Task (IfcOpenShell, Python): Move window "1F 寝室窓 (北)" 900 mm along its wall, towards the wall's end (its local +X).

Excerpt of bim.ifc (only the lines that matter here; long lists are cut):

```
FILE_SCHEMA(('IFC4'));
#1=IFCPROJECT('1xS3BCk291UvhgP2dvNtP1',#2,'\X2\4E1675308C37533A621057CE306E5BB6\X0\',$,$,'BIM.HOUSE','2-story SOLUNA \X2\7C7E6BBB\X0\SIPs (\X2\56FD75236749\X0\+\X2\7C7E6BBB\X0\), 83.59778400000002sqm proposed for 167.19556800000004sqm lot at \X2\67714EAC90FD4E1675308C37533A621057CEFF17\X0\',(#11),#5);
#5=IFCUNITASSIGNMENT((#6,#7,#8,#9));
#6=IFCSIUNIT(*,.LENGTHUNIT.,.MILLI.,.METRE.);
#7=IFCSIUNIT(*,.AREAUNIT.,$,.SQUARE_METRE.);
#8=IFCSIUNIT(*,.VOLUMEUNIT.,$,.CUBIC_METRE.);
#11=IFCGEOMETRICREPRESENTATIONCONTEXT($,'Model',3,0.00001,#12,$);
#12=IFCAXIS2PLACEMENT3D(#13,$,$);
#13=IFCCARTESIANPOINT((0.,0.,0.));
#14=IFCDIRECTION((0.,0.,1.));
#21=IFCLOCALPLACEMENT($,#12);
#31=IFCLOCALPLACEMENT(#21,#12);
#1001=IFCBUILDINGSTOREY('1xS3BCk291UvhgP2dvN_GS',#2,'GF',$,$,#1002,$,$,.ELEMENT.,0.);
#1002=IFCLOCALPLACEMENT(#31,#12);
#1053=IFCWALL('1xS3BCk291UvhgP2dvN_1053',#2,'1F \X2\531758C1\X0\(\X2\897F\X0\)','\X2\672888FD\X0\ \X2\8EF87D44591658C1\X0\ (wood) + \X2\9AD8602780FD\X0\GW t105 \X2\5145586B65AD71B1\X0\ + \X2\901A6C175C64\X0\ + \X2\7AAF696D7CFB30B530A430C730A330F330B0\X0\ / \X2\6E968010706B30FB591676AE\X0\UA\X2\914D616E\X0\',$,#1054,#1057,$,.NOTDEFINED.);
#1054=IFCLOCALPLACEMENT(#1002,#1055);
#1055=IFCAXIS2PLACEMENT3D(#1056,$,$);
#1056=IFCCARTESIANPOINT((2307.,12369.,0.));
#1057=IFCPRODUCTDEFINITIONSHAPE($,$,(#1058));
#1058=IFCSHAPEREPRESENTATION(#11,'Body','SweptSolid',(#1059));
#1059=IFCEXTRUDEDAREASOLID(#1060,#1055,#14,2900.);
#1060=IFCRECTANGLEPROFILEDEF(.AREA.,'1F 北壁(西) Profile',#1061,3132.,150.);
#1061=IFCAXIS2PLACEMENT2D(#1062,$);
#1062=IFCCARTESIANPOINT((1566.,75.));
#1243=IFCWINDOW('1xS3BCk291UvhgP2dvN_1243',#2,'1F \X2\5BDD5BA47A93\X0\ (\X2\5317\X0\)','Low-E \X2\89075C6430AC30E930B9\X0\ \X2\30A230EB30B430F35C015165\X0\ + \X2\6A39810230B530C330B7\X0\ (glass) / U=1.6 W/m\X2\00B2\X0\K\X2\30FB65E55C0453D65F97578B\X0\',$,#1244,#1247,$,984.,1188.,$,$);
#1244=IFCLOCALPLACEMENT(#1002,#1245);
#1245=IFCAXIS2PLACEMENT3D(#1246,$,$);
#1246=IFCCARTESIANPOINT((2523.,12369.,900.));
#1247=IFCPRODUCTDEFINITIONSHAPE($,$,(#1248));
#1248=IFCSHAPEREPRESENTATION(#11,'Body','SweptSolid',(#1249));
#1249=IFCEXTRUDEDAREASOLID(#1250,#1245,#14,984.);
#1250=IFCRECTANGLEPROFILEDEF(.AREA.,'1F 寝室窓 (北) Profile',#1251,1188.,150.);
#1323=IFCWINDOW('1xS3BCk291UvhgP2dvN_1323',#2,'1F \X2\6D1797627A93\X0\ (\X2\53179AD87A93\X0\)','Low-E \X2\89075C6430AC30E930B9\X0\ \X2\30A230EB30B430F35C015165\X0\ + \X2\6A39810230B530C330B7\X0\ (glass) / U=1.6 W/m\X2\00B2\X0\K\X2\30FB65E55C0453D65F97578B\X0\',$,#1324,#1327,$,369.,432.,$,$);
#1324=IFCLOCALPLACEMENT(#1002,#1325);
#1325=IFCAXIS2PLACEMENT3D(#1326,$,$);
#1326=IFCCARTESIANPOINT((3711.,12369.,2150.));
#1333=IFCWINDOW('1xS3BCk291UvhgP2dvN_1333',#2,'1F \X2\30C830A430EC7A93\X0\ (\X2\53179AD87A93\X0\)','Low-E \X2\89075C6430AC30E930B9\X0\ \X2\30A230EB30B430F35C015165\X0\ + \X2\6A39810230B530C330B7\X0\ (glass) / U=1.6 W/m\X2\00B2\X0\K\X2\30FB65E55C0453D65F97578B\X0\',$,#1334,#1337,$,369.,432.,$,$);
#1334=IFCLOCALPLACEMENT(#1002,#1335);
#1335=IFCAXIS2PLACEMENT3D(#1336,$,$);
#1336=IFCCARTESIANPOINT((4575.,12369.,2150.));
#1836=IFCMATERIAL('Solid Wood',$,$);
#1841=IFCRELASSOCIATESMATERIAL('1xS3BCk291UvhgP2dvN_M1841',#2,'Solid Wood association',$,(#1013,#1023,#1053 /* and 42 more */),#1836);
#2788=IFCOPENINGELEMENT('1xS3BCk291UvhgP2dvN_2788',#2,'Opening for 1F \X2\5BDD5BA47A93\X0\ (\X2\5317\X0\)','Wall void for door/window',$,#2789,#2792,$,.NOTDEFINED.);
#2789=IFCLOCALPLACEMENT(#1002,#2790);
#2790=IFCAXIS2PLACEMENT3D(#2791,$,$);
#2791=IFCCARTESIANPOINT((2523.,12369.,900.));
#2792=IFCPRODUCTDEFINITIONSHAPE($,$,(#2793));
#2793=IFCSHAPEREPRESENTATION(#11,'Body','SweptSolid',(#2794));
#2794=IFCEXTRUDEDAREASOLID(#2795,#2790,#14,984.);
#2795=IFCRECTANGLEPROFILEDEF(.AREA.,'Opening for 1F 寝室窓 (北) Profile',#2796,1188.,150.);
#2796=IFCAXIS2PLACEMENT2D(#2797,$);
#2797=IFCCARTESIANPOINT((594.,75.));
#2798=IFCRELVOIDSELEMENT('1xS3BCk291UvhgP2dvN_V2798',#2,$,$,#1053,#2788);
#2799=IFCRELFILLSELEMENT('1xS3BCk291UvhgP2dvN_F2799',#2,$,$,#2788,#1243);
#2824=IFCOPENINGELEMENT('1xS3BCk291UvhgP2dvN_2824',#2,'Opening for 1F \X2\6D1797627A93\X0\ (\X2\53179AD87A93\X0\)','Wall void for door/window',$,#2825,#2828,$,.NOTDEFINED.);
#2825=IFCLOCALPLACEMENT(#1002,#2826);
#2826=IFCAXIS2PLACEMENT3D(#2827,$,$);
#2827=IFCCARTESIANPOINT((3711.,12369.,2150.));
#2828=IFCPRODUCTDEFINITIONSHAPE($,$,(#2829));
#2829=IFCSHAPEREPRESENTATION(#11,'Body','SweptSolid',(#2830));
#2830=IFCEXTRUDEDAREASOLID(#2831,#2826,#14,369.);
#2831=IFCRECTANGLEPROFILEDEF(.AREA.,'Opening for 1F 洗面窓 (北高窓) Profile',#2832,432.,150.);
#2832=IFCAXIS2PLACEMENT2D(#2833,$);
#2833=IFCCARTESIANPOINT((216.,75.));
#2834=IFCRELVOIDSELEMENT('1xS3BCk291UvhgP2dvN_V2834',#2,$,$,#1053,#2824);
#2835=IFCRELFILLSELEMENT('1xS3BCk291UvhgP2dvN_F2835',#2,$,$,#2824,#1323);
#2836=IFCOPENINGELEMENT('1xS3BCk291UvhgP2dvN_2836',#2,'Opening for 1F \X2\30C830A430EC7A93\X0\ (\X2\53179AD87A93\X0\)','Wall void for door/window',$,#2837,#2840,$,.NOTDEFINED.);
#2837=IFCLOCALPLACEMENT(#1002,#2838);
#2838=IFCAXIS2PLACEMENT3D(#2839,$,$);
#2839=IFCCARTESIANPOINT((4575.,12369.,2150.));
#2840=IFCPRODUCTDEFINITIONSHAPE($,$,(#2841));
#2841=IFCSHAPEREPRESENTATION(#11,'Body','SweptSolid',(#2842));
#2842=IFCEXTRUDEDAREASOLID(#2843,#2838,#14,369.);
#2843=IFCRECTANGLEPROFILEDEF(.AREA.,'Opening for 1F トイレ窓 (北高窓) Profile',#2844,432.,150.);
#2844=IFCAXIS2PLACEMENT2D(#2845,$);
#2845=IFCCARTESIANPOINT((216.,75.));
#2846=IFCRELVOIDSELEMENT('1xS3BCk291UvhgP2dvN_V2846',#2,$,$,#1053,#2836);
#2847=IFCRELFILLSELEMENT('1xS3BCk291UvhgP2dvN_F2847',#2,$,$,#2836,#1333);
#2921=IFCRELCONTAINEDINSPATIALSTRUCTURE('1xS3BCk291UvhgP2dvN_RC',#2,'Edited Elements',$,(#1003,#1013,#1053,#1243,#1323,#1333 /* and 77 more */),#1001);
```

```python
import ifcopenshell
import ifcopenshell.api.geometry
import ifcopenshell.util.placement
import ifcopenshell.util.unit

model = ifcopenshell.open("bim.ifc")
unit_scale = ifcopenshell.util.unit.calculate_unit_scale(model)

window = model.by_guid("1xS3BCk291UvhgP2dvN_1243")
opening = window.FillsVoids[0].RelatingOpeningElement
wall = opening.VoidsElements[0].RelatingBuildingElement

wall_matrix = ifcopenshell.util.placement.get_local_placement(wall.ObjectPlacement)
shift = wall_matrix[:3, 0] * 0.9 / unit_scale
before = ifcopenshell.util.placement.get_local_placement(window.ObjectPlacement)[:3, 3].copy()

# The window is not placed relative to its opening, so move both.
for product in (opening, window):
    matrix = ifcopenshell.util.placement.get_local_placement(product.ObjectPlacement)
    matrix[:3, 3] += shift
    ifcopenshell.api.geometry.edit_object_placement(model, product=product, matrix=matrix, is_si=False)

after = ifcopenshell.util.placement.get_local_placement(window.ObjectPlacement)[:3, 3]
print("window moved by", (after - before).round(3) + 0.0)

model.write("bim_rev.ifc")
```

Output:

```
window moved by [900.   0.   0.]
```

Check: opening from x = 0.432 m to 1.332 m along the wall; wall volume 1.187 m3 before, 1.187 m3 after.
